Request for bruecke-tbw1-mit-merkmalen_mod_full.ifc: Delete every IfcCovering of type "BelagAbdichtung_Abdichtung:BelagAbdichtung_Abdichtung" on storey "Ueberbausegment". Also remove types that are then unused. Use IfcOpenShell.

First a look at what the model holds.

```python
import ifcopenshell
import ifcopenshell.util.element

model = ifcopenshell.open("bruecke-tbw1-mit-merkmalen_mod_full.ifc")
print(model.schema)
storey = next(s for s in model.by_type("IfcBuildingStorey") if s.Name == "Ueberbausegment")
coverings = [e for e in ifcopenshell.util.element.get_decomposition(storey) if e.is_a("IfcCovering")]
seen = {}
for e in coverings:
    element_type = ifcopenshell.util.element.get_type(e)
    name = element_type.Name if element_type not in (None, e) else None
    seen[name] = seen.get(name, 0) + 1
for name, count in sorted(seen.items(), key=str):
    print(count, "x", name)
```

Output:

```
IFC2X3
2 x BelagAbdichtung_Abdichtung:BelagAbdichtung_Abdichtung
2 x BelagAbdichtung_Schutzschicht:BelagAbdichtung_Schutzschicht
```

```python
import ifcopenshell
import ifcopenshell.api.root
import ifcopenshell.util.element

model = ifcopenshell.open("bruecke-tbw1-mit-merkmalen_mod_full.ifc")

storey = next(s for s in model.by_type("IfcBuildingStorey") if s.Name == "Ueberbausegment")
coverings = [e for e in ifcopenshell.util.element.get_decomposition(storey) if e.is_a("IfcCovering")]
targets = [e for e in coverings if (t := ifcopenshell.util.element.get_type(e)) not in (None, e) and t.Name == "BelagAbdichtung_Abdichtung:BelagAbdichtung_Abdichtung"]
types = {ifcopenshell.util.element.get_type(e) for e in targets} - {None, *targets}

for e in targets:
    ifcopenshell.api.root.remove_product(model, product=e)
print(len(targets), "removed")

unused = [t for t in types if not ifcopenshell.util.element.get_types(t)]
for t in unused:
    ifcopenshell.api.root.remove_product(model, product=t)
print(len(unused), "unused types removed")

model.write("bruecke-tbw1-mit-merkmalen_mod_full_rev.ifc")
```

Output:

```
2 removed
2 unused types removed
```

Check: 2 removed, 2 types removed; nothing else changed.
